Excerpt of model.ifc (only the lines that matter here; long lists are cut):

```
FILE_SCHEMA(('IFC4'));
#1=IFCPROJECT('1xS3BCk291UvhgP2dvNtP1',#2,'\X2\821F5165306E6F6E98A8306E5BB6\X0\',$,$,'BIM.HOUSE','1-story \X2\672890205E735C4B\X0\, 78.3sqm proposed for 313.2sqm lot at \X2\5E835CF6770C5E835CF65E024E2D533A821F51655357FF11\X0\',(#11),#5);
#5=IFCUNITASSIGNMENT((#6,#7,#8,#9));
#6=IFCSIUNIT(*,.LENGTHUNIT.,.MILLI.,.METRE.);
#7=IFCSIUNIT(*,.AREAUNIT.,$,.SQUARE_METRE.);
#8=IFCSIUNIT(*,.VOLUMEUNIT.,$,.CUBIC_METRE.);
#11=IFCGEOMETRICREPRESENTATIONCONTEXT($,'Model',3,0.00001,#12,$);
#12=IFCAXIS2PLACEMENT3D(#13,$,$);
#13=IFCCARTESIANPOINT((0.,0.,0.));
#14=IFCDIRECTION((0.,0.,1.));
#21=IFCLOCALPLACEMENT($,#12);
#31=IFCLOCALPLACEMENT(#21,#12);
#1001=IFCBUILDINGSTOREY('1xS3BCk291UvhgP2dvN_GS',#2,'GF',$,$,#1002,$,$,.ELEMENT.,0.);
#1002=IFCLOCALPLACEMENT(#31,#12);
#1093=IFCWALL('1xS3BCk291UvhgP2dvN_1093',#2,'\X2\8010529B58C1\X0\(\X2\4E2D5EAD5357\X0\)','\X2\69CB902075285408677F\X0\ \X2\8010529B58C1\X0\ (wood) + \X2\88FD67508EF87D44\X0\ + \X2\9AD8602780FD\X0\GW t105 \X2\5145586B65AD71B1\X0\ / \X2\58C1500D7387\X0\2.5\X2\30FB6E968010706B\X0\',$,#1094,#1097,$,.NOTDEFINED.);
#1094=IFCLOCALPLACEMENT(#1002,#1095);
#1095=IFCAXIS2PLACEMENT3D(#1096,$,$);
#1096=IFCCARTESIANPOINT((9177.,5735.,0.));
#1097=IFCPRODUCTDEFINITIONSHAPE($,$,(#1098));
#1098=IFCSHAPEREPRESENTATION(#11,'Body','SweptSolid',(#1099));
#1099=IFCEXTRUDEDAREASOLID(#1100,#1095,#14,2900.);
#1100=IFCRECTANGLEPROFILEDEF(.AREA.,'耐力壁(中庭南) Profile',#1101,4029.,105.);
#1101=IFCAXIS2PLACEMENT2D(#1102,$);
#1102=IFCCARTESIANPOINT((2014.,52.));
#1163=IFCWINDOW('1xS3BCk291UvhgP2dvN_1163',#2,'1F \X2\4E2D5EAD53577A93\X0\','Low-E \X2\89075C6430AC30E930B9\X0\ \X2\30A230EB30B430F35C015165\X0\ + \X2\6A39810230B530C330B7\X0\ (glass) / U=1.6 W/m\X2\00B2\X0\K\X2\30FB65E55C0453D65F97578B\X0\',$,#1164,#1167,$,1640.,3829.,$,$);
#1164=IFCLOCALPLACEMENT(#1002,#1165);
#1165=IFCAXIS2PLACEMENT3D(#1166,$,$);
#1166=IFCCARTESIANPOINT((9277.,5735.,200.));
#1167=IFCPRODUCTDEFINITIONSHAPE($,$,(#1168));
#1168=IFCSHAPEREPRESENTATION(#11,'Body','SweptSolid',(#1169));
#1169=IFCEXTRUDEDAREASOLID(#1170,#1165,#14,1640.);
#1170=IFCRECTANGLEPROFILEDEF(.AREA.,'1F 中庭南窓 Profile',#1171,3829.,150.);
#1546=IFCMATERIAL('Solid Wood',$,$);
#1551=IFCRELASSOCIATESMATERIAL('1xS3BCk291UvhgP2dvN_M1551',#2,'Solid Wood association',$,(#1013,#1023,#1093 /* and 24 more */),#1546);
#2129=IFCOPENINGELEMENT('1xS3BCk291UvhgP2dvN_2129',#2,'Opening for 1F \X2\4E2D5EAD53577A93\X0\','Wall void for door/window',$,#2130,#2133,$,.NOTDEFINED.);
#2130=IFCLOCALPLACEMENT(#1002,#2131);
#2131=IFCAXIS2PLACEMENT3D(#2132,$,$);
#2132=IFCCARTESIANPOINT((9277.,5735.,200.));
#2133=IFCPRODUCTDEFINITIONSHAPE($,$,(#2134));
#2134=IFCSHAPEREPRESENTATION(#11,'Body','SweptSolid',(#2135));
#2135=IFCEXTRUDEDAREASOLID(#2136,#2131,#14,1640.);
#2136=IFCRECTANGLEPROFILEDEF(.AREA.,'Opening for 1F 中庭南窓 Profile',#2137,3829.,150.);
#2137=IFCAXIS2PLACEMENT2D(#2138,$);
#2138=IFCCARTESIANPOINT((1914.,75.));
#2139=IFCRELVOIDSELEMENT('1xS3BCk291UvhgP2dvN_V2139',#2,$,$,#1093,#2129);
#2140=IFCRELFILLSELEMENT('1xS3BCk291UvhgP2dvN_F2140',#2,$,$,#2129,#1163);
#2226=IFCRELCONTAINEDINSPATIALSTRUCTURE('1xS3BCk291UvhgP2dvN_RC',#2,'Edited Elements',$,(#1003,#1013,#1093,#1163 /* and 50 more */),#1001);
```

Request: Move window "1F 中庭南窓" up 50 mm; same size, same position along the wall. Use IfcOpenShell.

```python
import numpy as np
import ifcopenshell
import ifcopenshell.api.geometry
import ifcopenshell.util.placement
import ifcopenshell.util.unit

model = ifcopenshell.open("model.ifc")
unit_scale = ifcopenshell.util.unit.calculate_unit_scale(model)

window = model.by_guid("1xS3BCk291UvhgP2dvN_1163")
opening = window.FillsVoids[0].RelatingOpeningElement
dz = 50.0

shift = np.array([0.0, 0.0, dz])
# The window is not placed relative to its opening, so move both.
for product in (opening, window):
    matrix = ifcopenshell.util.placement.get_local_placement(product.ObjectPlacement)
    matrix[:3, 3] += shift
    ifcopenshell.api.geometry.edit_object_placement(model, product=product, matrix=matrix, is_si=False)

print(f"moved by {dz * unit_scale:+.3f} m")

model.write("model-out.ifc")
```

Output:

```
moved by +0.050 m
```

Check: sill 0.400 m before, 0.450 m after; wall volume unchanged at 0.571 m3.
